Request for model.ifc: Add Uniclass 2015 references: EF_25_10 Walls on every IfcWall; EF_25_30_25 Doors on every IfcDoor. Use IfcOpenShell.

First a look at what the model holds.

```python
import ifcopenshell

model = ifcopenshell.open("model.ifc")
print(model.schema)
print("classifications:", [c.Name for c in model.by_type("IfcClassification")])
for ifc_class in ("IfcDoor", "IfcRoof", "IfcStair", "IfcWall", "IfcWindow"):
    print(ifc_class, len(model.by_type(ifc_class)))
```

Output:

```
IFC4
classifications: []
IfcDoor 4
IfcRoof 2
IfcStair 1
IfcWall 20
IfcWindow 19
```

```python
import ifcopenshell
import ifcopenshell.api.classification

model = ifcopenshell.open("model.ifc")

system = ifcopenshell.api.classification.add_classification(model, classification="Uniclass 2015")

codes = {
    "IfcWall": ("EF_25_10", "Walls"),
    "IfcDoor": ("EF_25_30_25", "Doors"),
}
for ifc_class, (code, name) in codes.items():
    products = model.by_type(ifc_class)
    ifcopenshell.api.classification.add_reference(
        model, products=products, classification=system, identification=code, name=name
    )
    print(code, len(products))

model.write("model_updated.ifc")
```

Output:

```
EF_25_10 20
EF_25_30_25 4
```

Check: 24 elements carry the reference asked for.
